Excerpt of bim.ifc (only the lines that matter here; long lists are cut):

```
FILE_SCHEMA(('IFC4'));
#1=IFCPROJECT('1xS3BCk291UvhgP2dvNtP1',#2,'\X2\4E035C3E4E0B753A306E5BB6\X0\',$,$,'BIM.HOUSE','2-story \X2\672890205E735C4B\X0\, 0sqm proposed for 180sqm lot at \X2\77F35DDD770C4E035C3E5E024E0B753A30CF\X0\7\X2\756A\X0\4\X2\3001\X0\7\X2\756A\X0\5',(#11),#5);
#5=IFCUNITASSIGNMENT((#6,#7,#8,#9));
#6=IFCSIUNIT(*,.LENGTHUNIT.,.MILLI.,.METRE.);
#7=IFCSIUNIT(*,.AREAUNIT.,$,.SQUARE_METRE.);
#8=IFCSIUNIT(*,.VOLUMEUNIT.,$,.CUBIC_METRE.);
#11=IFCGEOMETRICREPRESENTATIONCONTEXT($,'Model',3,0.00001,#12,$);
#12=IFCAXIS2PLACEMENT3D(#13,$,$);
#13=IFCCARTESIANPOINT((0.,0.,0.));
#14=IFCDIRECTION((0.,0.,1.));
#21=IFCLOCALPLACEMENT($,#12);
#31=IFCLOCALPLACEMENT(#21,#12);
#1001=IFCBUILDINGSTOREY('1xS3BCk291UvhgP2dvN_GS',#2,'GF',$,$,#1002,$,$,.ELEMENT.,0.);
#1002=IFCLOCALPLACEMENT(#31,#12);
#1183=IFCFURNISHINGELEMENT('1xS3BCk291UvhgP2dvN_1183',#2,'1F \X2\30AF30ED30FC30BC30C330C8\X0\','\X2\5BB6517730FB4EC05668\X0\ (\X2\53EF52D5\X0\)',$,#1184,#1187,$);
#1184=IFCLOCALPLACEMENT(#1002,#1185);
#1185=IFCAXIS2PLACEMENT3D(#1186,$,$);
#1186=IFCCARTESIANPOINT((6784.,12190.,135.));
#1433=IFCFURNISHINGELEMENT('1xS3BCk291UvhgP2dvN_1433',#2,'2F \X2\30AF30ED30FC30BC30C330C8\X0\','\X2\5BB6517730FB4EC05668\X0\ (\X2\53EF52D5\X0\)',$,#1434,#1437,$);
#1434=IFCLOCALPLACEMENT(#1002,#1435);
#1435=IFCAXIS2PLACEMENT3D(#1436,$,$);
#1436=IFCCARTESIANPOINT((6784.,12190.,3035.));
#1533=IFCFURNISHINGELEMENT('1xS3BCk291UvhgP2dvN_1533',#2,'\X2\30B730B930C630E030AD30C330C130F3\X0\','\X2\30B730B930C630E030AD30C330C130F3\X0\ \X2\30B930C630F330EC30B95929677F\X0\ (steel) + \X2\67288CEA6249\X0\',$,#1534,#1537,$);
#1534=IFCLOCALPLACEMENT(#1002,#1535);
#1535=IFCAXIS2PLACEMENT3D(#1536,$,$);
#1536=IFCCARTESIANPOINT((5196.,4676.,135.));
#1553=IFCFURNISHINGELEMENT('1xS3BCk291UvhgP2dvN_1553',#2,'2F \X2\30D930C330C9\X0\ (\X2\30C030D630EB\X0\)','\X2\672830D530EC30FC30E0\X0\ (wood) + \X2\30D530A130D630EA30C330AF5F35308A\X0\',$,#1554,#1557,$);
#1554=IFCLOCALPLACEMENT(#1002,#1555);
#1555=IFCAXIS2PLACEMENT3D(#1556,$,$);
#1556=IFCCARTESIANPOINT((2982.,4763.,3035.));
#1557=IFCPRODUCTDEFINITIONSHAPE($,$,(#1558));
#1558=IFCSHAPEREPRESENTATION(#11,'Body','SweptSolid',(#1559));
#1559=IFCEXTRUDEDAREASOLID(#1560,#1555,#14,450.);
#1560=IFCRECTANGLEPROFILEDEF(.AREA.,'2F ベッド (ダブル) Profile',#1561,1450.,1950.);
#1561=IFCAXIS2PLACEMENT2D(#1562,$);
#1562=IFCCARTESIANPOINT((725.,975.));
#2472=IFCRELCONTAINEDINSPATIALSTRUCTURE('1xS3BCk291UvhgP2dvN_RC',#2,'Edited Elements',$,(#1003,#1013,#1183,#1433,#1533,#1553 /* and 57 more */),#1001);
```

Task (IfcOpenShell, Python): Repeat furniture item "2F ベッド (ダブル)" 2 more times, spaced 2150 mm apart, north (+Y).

```python
import numpy as np
import ifcopenshell
import ifcopenshell.api.geometry
import ifcopenshell.api.root
import ifcopenshell.util.element
import ifcopenshell.util.placement
import ifcopenshell.util.unit

model = ifcopenshell.open("bim.ifc")
unit_scale = ifcopenshell.util.unit.calculate_unit_scale(model)


def reuse_history(source, copy):
    """copy_class also copies each property set's owner history, people and application; keep the originals."""
    for rel in copy.IsDefinedBy:
        if rel.is_a("IfcRelDefinesByProperties") and (history := rel.RelatingPropertyDefinition.OwnerHistory):
            rel.RelatingPropertyDefinition.OwnerHistory = source.OwnerHistory
            ifcopenshell.util.element.remove_deep2(model, history)


source = model.by_guid("1xS3BCk291UvhgP2dvN_1553")
base = ifcopenshell.util.placement.get_local_placement(source.ObjectPlacement)
step = np.array([0.0, 1.0, 0.0]) * 2.15 / unit_scale

for i in range(1, 3):
    copy = ifcopenshell.api.root.copy_class(model, product=source)
    copy.Representation = ifcopenshell.util.element.copy_deep(
        model, source.Representation, exclude=["IfcGeometricRepresentationContext", "IfcRepresentationMap"]
    )
    reuse_history(source, copy)
    matrix = base.copy()
    matrix[:3, 3] += i * step
    print("added at", matrix[:3, 3].round(3) + 0.0)
    ifcopenshell.api.geometry.edit_object_placement(model, product=copy, matrix=matrix, is_si=False)

model.write("bim-out.ifc")
```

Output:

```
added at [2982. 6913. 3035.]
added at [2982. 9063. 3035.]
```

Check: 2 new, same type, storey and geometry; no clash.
